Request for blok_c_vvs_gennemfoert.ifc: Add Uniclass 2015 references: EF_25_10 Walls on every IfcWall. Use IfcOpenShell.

First a look at what the model holds.

```python
import ifcopenshell

model = ifcopenshell.open("blok_c_vvs_gennemfoert.ifc")
print(model.schema)
print("classifications:", [c.Name for c in model.by_type("IfcClassification")])
for ifc_class in ("IfcDoor", "IfcRoof", "IfcStair", "IfcWall", "IfcWindow"):
    print(ifc_class, len(model.by_type(ifc_class)))
```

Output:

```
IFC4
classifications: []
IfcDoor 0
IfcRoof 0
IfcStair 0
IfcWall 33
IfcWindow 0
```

```python
import ifcopenshell
import ifcopenshell.api.classification

model = ifcopenshell.open("blok_c_vvs_gennemfoert.ifc")

system = ifcopenshell.api.classification.add_classification(model, classification="Uniclass 2015")

codes = {
    "IfcWall": ("EF_25_10", "Walls"),
}
for ifc_class, (code, name) in codes.items():
    products = model.by_type(ifc_class)
    ifcopenshell.api.classification.add_reference(
        model, products=products, classification=system, identification=code, name=name
    )
    print(code, len(products))

model.write("blok_c_vvs_gennemfoert_v2.ifc")
```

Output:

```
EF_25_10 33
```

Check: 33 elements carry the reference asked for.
